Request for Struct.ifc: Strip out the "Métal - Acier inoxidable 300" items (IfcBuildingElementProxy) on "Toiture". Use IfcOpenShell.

First a look at what the model holds.

```python
import ifcopenshell
import ifcopenshell.util.element

model = ifcopenshell.open("Struct.ifc")
print(model.schema)
storey = next(s for s in model.by_type("IfcBuildingStorey") if s.Name == "Toiture")
proxies = [e for e in ifcopenshell.util.element.get_decomposition(storey) if e.is_a("IfcBuildingElementProxy")]
seen = {}
for e in proxies:
    element_type = ifcopenshell.util.element.get_type(e)
    name = element_type.Name if element_type not in (None, e) else None
    seen[name] = seen.get(name, 0) + 1
for name, count in sorted(seen.items(), key=str):
    print(count, "x", name)
```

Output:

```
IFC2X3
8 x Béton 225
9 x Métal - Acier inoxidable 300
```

```python
import ifcopenshell
import ifcopenshell.api.root
import ifcopenshell.util.element

model = ifcopenshell.open("Struct.ifc")

storey = next(s for s in model.by_type("IfcBuildingStorey") if s.Name == "Toiture")
proxies = [e for e in ifcopenshell.util.element.get_decomposition(storey) if e.is_a("IfcBuildingElementProxy")]
targets = [e for e in proxies if (t := ifcopenshell.util.element.get_type(e)) not in (None, e) and t.Name == "Métal - Acier inoxidable 300"]

for e in targets:
    ifcopenshell.api.root.remove_product(model, product=e)
print(len(targets), "removed")

model.write("Struct_rev.ifc")
```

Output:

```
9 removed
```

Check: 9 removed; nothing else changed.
